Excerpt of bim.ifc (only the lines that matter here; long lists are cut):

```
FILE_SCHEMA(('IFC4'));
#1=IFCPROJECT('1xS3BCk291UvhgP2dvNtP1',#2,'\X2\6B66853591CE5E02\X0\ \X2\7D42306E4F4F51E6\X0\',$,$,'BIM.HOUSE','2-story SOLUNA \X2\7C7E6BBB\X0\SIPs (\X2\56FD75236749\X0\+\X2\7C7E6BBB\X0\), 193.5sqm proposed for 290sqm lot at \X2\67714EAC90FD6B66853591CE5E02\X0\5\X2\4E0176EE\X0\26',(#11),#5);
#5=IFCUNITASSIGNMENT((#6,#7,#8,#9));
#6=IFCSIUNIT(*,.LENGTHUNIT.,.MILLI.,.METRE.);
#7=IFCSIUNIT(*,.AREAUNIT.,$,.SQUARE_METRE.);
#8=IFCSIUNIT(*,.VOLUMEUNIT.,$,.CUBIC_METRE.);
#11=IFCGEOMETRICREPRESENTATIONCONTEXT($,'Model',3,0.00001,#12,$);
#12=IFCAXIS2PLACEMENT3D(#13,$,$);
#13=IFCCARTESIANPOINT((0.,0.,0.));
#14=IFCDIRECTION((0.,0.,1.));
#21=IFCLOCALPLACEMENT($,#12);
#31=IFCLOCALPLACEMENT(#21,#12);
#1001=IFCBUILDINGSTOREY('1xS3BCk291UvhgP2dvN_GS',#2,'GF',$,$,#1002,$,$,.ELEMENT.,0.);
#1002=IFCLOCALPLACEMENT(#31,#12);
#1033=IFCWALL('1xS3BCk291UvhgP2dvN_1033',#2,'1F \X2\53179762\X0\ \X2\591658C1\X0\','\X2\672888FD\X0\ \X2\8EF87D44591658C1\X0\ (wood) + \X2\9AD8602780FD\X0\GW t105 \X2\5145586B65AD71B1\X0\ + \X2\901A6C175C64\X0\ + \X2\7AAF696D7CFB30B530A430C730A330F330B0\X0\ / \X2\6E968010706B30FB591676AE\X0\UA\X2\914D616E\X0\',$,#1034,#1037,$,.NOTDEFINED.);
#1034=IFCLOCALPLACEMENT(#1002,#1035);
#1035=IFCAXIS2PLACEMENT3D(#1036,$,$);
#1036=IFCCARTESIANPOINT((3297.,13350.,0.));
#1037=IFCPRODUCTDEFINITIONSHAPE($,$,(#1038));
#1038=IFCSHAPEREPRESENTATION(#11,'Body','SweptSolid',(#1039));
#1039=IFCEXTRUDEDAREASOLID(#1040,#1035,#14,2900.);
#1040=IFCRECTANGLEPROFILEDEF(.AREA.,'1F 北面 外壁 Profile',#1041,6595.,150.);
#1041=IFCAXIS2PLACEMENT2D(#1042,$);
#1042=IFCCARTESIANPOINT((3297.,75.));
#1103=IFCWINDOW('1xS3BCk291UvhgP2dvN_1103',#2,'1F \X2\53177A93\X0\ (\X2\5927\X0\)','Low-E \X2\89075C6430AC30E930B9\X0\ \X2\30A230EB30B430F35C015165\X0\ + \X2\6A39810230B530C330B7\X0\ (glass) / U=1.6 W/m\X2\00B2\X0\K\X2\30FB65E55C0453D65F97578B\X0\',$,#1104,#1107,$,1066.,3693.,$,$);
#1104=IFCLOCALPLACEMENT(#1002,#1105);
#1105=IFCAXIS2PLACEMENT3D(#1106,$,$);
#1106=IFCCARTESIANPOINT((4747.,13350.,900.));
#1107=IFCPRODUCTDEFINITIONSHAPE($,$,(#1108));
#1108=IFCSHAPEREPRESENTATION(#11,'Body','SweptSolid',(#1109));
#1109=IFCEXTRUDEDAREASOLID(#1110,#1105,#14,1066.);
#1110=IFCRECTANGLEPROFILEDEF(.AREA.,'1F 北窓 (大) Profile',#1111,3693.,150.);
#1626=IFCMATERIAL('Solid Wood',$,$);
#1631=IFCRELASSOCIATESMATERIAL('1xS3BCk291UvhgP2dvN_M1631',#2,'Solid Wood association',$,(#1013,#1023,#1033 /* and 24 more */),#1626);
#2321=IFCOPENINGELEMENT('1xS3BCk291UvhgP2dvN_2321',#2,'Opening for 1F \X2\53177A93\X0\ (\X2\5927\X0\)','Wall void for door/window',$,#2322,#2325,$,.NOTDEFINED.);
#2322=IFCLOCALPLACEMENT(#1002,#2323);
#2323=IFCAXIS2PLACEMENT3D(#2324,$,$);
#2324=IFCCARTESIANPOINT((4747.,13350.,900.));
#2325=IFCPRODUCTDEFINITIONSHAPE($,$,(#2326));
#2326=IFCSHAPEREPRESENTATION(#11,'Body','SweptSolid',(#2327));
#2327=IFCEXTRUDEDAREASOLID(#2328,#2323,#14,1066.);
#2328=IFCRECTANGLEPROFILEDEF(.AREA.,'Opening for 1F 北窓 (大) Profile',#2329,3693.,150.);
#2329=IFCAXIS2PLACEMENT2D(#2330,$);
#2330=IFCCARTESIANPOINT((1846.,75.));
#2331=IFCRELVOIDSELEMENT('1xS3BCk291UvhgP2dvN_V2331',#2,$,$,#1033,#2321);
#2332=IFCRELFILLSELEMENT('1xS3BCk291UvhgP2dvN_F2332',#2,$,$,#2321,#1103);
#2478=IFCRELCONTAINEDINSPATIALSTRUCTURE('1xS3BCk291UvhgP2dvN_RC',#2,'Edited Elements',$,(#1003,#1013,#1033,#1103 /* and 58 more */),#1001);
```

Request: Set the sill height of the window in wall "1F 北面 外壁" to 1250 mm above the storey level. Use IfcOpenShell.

```python
import numpy as np
import ifcopenshell
import ifcopenshell.api.geometry
import ifcopenshell.geom
import ifcopenshell.util.element
import ifcopenshell.util.placement
import ifcopenshell.util.shape
import ifcopenshell.util.unit

model = ifcopenshell.open("bim.ifc")
unit_scale = ifcopenshell.util.unit.calculate_unit_scale(model)

window = model.by_id(1103)
opening = window.FillsVoids[0].RelatingOpeningElement
storey = ifcopenshell.util.element.get_container(window, ifc_class="IfcBuildingStorey")
level = ifcopenshell.util.placement.get_local_placement(storey.ObjectPlacement)[2, 3]

# The opening's origin need not be at the sill, so measure its lowest point.
shape = ifcopenshell.geom.create_shape(ifcopenshell.geom.settings(), opening)
bottom = ifcopenshell.util.shape.get_shape_bottom_elevation(shape, shape.geometry) / unit_scale
dz = level + 1250.0 - bottom

shift = np.array([0.0, 0.0, dz])
# The window is not placed relative to its opening, so move both.
for product in (opening, window):
    matrix = ifcopenshell.util.placement.get_local_placement(product.ObjectPlacement)
    matrix[:3, 3] += shift
    ifcopenshell.api.geometry.edit_object_placement(model, product=product, matrix=matrix, is_si=False)

print(f"moved by {dz * unit_scale:+.3f} m")

model.write("bim_updated.ifc")
```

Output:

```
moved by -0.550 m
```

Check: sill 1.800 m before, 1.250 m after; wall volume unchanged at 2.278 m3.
